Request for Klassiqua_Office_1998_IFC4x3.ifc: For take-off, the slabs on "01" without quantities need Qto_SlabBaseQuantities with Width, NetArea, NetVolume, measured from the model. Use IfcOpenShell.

First a look at what the model holds.

```python
import ifcopenshell
import ifcopenshell.util.element
import ifcopenshell.util.unit

model = ifcopenshell.open("Klassiqua_Office_1998_IFC4x3.ifc")
print(model.schema)
for unit_type in ("LENGTHUNIT", "AREAUNIT", "VOLUMEUNIT"):
    print(unit_type, ifcopenshell.util.unit.calculate_unit_scale(model, unit_type))
storey = next(s for s in model.by_type("IfcBuildingStorey") if s.Name == "01")
slabs = [e for e in ifcopenshell.util.element.get_decomposition(storey) if e.is_a("IfcSlab")]
for e in sorted(slabs, key=lambda e: e.id()):
    print(e.id(), e.is_a(), e.Name, list(ifcopenshell.util.element.get_psets(e, qtos_only=True)), sep=" | ")
```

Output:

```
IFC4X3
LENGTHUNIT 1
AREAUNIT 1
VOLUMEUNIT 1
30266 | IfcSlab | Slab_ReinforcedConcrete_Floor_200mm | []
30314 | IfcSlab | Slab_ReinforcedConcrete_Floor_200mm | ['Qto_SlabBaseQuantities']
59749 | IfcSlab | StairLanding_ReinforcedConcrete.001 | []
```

```python
import ifcopenshell
import ifcopenshell.api.pset
import ifcopenshell.geom
import ifcopenshell.util.element
import ifcopenshell.util.shape
import ifcopenshell.util.unit

model = ifcopenshell.open("Klassiqua_Office_1998_IFC4x3.ifc")
unit_scale = ifcopenshell.util.unit.calculate_unit_scale(model)
area_scale = ifcopenshell.util.unit.calculate_unit_scale(model, "AREAUNIT")
volume_scale = ifcopenshell.util.unit.calculate_unit_scale(model, "VOLUMEUNIT")
settings = ifcopenshell.geom.settings()

storey = next(s for s in model.by_type("IfcBuildingStorey") if s.Name == "01")
slabs = [e for e in ifcopenshell.util.element.get_decomposition(storey) if e.is_a("IfcSlab")]

for e in sorted(slabs, key=lambda e: e.id()):
    if ifcopenshell.util.element.get_psets(e, qtos_only=True, should_inherit=False):
        continue
    # Geometry comes back in metres, in the element's own axes.
    shape = ifcopenshell.geom.create_shape(settings, e)
    values = {
        "Width": ifcopenshell.util.shape.get_z(shape.geometry) / unit_scale,
        "NetArea": ifcopenshell.util.shape.get_footprint_area(shape.geometry) / area_scale,
        "NetVolume": ifcopenshell.util.shape.get_volume(shape.geometry) / volume_scale,
    }
    qto = ifcopenshell.api.pset.add_qto(model, product=e, name="Qto_SlabBaseQuantities")
    ifcopenshell.api.pset.edit_qto(model, qto=qto, properties=values)
    print(e.id(), {k: round(v, 3) for k, v in values.items()})

model.write("Klassiqua_Office_1998_IFC4x3_v2.ifc")
```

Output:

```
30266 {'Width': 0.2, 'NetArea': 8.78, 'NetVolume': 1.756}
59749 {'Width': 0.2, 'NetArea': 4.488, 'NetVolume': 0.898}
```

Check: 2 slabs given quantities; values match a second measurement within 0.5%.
